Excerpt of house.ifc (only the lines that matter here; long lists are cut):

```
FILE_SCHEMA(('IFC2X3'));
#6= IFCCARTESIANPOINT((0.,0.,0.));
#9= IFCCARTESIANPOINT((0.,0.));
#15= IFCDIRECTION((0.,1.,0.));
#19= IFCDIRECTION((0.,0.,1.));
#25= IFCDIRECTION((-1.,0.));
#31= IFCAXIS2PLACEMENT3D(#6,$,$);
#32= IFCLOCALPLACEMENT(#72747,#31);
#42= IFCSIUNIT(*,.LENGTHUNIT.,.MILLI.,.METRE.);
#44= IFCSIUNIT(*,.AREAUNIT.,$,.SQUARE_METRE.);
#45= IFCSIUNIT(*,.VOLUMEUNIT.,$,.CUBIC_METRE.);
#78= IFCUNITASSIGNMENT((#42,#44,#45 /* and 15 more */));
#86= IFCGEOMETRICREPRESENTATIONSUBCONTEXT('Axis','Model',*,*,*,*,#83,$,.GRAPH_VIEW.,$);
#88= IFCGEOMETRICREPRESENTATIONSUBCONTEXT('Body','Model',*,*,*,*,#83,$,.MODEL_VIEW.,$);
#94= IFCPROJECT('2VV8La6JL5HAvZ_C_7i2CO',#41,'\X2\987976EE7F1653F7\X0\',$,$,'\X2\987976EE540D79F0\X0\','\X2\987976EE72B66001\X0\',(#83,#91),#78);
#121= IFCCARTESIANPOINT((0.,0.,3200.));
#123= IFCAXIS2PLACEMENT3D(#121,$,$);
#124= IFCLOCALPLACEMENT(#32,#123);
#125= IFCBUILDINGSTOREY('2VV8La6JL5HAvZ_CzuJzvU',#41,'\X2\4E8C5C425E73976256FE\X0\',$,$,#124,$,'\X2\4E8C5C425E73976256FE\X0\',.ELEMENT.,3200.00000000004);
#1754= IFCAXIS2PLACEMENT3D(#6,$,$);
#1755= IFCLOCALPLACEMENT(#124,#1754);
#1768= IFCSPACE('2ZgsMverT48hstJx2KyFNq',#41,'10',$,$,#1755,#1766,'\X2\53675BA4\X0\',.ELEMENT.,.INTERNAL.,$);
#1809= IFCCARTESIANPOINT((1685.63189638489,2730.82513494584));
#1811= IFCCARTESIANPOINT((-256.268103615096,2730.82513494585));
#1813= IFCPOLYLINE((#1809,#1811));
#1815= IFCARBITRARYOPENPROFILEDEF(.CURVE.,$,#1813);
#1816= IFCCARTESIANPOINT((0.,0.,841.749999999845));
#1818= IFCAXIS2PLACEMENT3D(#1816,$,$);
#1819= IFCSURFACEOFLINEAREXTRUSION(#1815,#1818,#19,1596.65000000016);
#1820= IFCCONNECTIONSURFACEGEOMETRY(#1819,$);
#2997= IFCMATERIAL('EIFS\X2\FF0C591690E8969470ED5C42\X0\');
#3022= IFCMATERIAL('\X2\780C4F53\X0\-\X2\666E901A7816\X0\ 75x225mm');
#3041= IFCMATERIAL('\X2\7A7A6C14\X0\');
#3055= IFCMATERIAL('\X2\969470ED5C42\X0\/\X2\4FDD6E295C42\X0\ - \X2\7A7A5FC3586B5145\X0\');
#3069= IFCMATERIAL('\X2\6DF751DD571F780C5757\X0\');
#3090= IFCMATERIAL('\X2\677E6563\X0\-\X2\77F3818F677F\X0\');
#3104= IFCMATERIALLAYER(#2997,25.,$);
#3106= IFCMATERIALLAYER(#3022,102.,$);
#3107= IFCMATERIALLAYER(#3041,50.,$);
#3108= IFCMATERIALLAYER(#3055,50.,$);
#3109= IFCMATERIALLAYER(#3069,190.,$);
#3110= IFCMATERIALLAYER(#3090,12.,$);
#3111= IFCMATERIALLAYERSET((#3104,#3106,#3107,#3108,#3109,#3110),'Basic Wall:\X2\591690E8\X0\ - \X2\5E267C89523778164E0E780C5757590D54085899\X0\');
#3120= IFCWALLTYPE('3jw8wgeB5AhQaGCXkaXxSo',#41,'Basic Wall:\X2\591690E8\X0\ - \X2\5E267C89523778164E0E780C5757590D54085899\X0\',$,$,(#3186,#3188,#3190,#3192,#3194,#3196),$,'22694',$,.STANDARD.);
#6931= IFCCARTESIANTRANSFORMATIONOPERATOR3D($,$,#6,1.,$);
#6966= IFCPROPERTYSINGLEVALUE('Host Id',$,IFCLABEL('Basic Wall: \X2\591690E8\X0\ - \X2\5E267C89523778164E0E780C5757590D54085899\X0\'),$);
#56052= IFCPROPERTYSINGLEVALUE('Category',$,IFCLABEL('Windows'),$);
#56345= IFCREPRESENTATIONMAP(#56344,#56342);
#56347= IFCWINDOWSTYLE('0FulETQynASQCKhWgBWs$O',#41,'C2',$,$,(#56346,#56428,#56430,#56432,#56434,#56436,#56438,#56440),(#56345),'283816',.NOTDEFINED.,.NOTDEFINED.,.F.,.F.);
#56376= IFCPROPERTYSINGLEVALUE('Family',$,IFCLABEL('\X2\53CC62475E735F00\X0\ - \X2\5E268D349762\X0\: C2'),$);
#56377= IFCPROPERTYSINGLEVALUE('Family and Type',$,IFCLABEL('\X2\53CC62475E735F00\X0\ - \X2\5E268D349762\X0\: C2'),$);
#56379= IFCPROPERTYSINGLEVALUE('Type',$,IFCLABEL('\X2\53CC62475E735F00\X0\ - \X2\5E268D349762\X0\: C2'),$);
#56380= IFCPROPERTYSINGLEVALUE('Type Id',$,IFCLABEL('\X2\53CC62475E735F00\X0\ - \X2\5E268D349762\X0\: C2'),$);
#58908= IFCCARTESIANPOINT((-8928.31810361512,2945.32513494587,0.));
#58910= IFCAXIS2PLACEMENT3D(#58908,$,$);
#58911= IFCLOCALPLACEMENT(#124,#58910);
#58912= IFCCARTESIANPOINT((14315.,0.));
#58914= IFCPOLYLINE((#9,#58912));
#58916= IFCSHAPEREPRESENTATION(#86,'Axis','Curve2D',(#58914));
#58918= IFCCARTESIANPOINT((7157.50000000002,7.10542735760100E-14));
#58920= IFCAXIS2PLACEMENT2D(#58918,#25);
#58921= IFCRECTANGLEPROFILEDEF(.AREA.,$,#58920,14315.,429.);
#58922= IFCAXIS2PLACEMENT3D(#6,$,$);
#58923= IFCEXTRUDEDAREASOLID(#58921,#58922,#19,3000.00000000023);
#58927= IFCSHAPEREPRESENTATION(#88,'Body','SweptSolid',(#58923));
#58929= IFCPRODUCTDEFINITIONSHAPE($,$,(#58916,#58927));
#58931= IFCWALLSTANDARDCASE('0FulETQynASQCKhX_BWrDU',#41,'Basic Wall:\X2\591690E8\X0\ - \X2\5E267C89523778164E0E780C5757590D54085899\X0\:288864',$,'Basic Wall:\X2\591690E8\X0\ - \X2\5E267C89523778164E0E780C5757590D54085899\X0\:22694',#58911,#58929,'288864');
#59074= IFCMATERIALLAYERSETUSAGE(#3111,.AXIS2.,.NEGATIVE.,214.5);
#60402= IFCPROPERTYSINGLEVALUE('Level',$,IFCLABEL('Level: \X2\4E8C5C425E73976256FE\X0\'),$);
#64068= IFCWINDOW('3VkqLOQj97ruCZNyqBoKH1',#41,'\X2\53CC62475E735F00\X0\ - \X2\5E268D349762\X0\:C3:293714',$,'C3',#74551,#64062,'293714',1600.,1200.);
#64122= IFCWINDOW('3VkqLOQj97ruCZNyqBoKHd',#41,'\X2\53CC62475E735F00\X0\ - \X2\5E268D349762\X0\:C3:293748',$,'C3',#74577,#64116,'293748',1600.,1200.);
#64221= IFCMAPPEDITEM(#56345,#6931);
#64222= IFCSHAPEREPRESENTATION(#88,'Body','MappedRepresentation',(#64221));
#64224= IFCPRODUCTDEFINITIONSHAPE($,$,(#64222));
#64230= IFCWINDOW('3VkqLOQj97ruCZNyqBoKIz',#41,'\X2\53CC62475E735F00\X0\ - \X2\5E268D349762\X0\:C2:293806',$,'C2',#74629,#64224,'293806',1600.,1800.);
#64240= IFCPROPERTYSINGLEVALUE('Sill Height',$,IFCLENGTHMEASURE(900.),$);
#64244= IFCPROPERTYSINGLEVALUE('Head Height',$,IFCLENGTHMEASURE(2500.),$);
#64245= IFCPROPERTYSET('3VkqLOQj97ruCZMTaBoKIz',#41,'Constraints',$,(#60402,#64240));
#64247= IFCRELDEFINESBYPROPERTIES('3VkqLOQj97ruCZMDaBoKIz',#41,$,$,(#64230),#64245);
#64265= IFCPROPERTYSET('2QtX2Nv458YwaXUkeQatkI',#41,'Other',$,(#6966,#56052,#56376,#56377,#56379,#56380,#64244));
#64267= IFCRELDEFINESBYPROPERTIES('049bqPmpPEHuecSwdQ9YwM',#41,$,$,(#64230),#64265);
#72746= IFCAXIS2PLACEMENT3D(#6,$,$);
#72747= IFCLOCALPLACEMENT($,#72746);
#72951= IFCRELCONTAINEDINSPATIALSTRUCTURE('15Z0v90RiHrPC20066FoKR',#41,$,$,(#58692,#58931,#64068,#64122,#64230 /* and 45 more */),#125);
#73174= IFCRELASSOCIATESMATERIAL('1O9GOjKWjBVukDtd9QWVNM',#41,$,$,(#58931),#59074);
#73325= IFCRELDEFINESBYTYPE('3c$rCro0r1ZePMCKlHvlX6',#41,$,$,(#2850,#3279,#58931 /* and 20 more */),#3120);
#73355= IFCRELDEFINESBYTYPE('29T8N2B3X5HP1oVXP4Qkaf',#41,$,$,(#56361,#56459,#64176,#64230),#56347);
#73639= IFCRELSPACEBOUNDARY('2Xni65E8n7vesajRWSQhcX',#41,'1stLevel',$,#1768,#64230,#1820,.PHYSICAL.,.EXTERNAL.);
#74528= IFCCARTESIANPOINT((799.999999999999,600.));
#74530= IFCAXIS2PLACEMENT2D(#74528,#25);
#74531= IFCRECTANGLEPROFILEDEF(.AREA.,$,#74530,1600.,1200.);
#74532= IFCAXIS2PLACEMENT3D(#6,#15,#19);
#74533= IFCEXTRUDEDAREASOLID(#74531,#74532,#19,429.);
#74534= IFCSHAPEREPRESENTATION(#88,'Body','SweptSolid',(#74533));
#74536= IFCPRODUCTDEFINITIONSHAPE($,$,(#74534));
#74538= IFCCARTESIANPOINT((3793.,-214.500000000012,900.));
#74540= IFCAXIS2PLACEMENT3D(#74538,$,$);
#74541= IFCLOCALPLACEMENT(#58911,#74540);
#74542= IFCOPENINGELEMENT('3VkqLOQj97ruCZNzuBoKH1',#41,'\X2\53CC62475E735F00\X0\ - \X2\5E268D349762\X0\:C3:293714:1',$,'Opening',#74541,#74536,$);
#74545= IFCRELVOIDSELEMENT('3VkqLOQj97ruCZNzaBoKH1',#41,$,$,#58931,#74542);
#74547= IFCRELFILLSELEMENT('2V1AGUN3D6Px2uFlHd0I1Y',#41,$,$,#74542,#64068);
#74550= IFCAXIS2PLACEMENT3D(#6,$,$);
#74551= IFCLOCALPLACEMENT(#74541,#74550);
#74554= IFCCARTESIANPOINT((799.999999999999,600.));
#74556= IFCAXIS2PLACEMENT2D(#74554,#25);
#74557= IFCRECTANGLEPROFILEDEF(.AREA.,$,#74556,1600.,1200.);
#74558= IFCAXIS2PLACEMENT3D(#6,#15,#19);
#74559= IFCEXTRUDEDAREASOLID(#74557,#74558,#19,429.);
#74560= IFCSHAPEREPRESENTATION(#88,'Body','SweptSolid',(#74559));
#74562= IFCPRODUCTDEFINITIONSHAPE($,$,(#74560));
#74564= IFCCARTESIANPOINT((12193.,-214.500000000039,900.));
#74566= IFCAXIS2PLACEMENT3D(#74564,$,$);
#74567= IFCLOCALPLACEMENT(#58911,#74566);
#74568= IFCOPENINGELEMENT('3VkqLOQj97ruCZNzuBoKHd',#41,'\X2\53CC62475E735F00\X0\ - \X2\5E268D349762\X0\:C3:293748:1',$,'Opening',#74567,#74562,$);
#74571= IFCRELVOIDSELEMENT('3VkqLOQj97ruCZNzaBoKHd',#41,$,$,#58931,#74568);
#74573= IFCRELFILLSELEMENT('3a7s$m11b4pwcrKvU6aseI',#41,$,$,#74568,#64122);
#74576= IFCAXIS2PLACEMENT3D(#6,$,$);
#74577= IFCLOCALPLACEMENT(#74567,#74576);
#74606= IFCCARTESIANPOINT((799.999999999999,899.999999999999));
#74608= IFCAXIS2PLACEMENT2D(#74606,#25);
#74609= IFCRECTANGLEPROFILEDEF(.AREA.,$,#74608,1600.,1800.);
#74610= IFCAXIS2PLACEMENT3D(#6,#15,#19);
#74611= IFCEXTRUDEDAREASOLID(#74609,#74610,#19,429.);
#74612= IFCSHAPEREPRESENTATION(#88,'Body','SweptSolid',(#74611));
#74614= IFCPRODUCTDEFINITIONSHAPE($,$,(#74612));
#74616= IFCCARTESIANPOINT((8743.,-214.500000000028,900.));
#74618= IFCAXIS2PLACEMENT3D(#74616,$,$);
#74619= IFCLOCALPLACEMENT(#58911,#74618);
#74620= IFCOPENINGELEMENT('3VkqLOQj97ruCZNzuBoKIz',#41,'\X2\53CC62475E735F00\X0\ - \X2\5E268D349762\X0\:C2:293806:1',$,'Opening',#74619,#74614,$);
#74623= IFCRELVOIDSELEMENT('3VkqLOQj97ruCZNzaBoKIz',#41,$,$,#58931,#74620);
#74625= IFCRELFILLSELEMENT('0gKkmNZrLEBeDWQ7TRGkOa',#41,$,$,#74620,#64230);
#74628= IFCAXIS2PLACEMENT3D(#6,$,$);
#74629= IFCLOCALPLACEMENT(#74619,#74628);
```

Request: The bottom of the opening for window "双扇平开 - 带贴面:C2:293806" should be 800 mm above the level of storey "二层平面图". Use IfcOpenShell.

```python
import numpy as np
import ifcopenshell
import ifcopenshell.api.geometry
import ifcopenshell.api.pset
import ifcopenshell.geom
import ifcopenshell.util.element
import ifcopenshell.util.placement
import ifcopenshell.util.shape
import ifcopenshell.util.unit

model = ifcopenshell.open("house.ifc")
unit_scale = ifcopenshell.util.unit.calculate_unit_scale(model)

window = model.by_guid("3VkqLOQj97ruCZNyqBoKIz")
opening = window.FillsVoids[0].RelatingOpeningElement
storey = ifcopenshell.util.element.get_container(window, ifc_class="IfcBuildingStorey")
level = ifcopenshell.util.placement.get_local_placement(storey.ObjectPlacement)[2, 3]

# The opening's origin need not be at the sill, so measure its lowest point.
shape = ifcopenshell.geom.create_shape(ifcopenshell.geom.settings(), opening)
bottom = ifcopenshell.util.shape.get_shape_bottom_elevation(shape, shape.geometry) / unit_scale
dz = level + 800.0 - bottom

shift = np.array([0.0, 0.0, dz])
# The window is placed relative to its opening, so it follows when the opening moves.
matrix = ifcopenshell.util.placement.get_local_placement(opening.ObjectPlacement)
matrix[:3, 3] += shift
ifcopenshell.api.geometry.edit_object_placement(
    model, product=opening, matrix=matrix, is_si=False, should_transform_children=True
)

# Space boundary surfaces are stored in each space's coordinates; move them too.
for rel in window.ProvidesBoundaries:
    if not rel.ConnectionGeometry:
        continue
    surface = rel.ConnectionGeometry.SurfaceOnRelatingElement
    space_matrix = ifcopenshell.util.placement.get_local_placement(rel.RelatingSpace.ObjectPlacement)
    point = np.array(surface.Position.Location.Coordinates) + space_matrix[:3, :3].T @ shift
    surface.Position = model.createIfcAxis2Placement3D(
        model.createIfcCartesianPoint(point.tolist()), surface.Position.Axis, surface.Position.RefDirection
    )

# Keep the stored heights in step.
pset = model.by_id(ifcopenshell.util.element.get_pset(window, "Constraints", should_inherit=False)["id"])
ifcopenshell.api.pset.edit_pset(model, pset=pset, properties={
    "Sill Height": model.create_entity("IfcLengthMeasure", ifcopenshell.util.element.get_pset(window, "Constraints", "Sill Height") + dz),
})
pset = model.by_id(ifcopenshell.util.element.get_pset(window, "Other", should_inherit=False)["id"])
ifcopenshell.api.pset.edit_pset(model, pset=pset, properties={
    "Head Height": model.create_entity("IfcLengthMeasure", ifcopenshell.util.element.get_pset(window, "Other", "Head Height") + dz),
})

print(f"moved by {dz * unit_scale:+.3f} m")

model.write("house_updated.ifc")
```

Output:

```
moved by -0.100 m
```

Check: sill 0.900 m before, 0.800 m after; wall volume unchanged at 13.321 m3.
